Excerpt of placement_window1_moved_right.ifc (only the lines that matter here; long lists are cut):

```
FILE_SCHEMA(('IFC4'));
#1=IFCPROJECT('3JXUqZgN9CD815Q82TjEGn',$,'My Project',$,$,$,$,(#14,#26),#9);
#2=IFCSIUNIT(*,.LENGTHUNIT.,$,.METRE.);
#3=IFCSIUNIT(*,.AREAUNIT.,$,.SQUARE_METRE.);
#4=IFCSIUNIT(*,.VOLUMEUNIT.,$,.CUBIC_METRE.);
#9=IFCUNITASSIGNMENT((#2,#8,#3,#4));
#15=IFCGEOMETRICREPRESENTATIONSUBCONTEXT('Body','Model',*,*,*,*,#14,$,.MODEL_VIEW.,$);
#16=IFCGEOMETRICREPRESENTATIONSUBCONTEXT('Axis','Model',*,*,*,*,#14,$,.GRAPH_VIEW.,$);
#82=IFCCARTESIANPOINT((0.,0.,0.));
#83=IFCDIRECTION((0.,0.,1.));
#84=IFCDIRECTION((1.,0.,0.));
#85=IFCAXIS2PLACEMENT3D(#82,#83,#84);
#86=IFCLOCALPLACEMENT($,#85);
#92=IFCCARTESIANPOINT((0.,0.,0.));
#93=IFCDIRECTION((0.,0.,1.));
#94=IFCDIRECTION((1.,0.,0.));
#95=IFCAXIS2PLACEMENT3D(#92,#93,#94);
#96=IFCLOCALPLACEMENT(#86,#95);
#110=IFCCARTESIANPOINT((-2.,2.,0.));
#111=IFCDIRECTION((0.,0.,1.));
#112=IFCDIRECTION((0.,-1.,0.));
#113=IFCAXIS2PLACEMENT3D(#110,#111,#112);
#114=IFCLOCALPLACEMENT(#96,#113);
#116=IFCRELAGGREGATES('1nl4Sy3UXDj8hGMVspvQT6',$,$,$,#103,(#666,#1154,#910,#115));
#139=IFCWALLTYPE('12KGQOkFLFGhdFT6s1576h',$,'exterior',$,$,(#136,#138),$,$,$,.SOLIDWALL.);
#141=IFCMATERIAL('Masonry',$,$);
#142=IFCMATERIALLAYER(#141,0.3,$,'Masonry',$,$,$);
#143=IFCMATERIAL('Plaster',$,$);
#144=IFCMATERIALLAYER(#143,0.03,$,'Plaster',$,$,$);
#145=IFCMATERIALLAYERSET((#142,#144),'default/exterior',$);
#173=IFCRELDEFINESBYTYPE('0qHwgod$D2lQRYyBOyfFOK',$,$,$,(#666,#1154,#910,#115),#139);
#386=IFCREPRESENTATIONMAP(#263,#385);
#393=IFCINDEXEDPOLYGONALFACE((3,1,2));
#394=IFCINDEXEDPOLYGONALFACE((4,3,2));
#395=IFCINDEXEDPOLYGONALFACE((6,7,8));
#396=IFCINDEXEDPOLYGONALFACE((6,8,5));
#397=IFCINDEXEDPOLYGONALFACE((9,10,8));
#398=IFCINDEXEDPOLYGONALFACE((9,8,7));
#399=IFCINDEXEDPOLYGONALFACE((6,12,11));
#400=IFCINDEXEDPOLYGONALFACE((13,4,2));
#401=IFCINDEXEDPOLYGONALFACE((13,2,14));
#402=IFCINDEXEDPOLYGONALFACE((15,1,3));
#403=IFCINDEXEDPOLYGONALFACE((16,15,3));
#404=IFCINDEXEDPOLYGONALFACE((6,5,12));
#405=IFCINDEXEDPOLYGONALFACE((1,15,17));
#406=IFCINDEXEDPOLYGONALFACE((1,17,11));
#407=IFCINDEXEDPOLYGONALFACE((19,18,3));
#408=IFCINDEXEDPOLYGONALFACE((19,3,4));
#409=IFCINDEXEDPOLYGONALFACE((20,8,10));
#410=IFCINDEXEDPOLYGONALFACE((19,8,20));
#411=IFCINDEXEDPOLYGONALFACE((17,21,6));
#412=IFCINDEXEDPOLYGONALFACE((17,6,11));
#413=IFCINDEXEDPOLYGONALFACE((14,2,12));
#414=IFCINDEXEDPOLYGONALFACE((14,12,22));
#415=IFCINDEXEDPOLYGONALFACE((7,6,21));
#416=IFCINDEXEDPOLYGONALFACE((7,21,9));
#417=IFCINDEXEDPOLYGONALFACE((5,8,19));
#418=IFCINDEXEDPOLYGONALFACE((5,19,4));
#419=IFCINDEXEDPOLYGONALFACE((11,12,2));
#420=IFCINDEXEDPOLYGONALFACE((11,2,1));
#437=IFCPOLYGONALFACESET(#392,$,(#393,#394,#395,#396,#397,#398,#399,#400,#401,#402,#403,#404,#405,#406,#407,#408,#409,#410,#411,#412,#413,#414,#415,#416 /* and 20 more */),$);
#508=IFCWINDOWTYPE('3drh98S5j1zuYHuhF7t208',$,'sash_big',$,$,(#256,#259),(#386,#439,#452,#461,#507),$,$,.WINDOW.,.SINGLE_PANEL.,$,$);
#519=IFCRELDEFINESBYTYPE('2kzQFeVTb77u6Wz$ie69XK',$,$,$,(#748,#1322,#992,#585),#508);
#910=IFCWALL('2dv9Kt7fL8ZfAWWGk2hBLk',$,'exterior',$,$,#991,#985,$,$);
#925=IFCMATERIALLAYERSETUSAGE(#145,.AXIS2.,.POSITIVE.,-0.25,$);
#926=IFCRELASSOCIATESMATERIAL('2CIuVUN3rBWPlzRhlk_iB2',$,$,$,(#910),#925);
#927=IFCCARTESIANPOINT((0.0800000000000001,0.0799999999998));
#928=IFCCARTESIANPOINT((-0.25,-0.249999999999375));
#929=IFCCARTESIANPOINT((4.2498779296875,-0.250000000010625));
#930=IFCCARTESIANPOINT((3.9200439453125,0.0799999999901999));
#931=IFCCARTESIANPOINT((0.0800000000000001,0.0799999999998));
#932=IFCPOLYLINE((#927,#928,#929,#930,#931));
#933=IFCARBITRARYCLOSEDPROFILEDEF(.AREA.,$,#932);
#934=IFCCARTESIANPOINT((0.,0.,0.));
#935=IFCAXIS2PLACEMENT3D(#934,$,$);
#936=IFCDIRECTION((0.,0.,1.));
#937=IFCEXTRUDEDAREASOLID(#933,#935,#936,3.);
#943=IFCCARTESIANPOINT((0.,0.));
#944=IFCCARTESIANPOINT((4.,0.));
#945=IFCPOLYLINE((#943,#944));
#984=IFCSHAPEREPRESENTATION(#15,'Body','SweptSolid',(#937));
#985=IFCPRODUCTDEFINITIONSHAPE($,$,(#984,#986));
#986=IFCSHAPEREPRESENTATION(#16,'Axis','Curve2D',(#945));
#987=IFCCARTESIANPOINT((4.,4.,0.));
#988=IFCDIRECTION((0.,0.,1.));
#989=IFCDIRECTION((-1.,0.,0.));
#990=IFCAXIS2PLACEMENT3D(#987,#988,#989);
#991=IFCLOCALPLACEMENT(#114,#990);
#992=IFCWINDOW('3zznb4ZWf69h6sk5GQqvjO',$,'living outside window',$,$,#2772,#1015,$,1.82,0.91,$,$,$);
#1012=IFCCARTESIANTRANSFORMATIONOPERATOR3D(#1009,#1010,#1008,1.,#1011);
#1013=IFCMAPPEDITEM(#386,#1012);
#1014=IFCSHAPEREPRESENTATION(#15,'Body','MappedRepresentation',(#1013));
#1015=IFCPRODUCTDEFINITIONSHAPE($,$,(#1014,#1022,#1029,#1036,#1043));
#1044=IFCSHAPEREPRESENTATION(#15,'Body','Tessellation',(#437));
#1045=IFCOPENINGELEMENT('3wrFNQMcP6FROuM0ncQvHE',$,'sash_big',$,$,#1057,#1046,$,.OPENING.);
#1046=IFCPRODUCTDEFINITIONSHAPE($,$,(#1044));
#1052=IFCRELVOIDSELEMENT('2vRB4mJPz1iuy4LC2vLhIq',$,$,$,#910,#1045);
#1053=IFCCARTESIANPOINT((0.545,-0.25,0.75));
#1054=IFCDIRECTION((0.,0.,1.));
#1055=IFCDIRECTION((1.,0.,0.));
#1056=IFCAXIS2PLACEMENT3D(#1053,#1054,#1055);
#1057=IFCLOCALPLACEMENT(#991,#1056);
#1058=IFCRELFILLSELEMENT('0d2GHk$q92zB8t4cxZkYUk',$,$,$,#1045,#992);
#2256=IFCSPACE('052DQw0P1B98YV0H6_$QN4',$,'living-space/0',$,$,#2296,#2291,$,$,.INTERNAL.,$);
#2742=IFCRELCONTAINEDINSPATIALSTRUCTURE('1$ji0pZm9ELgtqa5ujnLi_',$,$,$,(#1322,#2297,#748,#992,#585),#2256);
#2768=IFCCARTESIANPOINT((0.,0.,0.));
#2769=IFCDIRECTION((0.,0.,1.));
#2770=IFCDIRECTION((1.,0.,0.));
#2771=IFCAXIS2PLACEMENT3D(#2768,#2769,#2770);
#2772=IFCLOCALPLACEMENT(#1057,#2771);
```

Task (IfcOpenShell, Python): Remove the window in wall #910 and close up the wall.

```python
import ifcopenshell
import ifcopenshell.api.feature
import ifcopenshell.api.root
import ifcopenshell.geom
import ifcopenshell.util.shape

model = ifcopenshell.open("placement_window1_moved_right.ifc")
settings = ifcopenshell.geom.settings()


def volume(element):
    """Net volume in cubic metres, openings subtracted."""
    shape = ifcopenshell.geom.create_shape(settings, element)
    return ifcopenshell.util.shape.get_volume(shape.geometry)


window = model.by_guid("3zznb4ZWf69h6sk5GQqvjO")
opening = window.FillsVoids[0].RelatingOpeningElement
wall = opening.VoidsElements[0].RelatingBuildingElement
before = volume(wall)

ifcopenshell.api.root.remove_product(model, product=window)
ifcopenshell.api.feature.remove_feature(model, feature=opening)

after = volume(wall)

print(f"wall volume {before:.3f} -> {after:.3f} m3")

model.write("placement_window1_moved_right_edited.ifc")
```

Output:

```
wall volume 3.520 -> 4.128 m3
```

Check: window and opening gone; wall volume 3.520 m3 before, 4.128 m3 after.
